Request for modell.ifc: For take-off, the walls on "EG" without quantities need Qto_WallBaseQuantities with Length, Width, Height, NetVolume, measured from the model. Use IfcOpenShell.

First a look at what the model holds.

```python
import ifcopenshell
import ifcopenshell.util.element
import ifcopenshell.util.unit

model = ifcopenshell.open("modell.ifc")
print(model.schema)
for unit_type in ("LENGTHUNIT", "AREAUNIT", "VOLUMEUNIT"):
    print(unit_type, ifcopenshell.util.unit.calculate_unit_scale(model, unit_type))
storey = next(s for s in model.by_type("IfcBuildingStorey") if s.Name == "EG")
walls = [e for e in ifcopenshell.util.element.get_decomposition(storey) if e.is_a("IfcWall")]
for e in sorted(walls, key=lambda e: e.id()):
    print(e.id(), e.is_a(), e.Name, list(ifcopenshell.util.element.get_psets(e, qtos_only=True)), sep=" | ")
```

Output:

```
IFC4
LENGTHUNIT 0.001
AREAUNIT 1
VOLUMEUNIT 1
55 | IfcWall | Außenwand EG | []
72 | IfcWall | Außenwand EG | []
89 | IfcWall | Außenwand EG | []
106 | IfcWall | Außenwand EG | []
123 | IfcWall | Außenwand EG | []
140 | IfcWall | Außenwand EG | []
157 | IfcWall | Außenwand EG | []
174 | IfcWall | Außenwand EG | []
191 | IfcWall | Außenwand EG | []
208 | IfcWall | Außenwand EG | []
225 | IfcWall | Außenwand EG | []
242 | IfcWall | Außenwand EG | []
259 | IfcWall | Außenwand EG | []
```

```python
import ifcopenshell
import ifcopenshell.api.pset
import ifcopenshell.geom
import ifcopenshell.util.element
import ifcopenshell.util.shape
import ifcopenshell.util.unit

model = ifcopenshell.open("modell.ifc")
unit_scale = ifcopenshell.util.unit.calculate_unit_scale(model)
volume_scale = ifcopenshell.util.unit.calculate_unit_scale(model, "VOLUMEUNIT")
settings = ifcopenshell.geom.settings()

storey = next(s for s in model.by_type("IfcBuildingStorey") if s.Name == "EG")
walls = [e for e in ifcopenshell.util.element.get_decomposition(storey) if e.is_a("IfcWall")]

for e in sorted(walls, key=lambda e: e.id()):
    if ifcopenshell.util.element.get_psets(e, qtos_only=True, should_inherit=False):
        continue
    # Geometry comes back in metres, in the element's own axes.
    shape = ifcopenshell.geom.create_shape(settings, e)
    values = {
        "Length": ifcopenshell.util.shape.get_x(shape.geometry) / unit_scale,
        "Width": ifcopenshell.util.shape.get_y(shape.geometry) / unit_scale,
        "Height": ifcopenshell.util.shape.get_z(shape.geometry) / unit_scale,
        "NetVolume": ifcopenshell.util.shape.get_volume(shape.geometry) / volume_scale,
    }
    qto = ifcopenshell.api.pset.add_qto(model, product=e, name="Qto_WallBaseQuantities")
    ifcopenshell.api.pset.edit_qto(model, qto=qto, properties=values)
    print(e.id(), {k: round(v, 3) for k, v in values.items()})

model.write("modell_rev.ifc")
```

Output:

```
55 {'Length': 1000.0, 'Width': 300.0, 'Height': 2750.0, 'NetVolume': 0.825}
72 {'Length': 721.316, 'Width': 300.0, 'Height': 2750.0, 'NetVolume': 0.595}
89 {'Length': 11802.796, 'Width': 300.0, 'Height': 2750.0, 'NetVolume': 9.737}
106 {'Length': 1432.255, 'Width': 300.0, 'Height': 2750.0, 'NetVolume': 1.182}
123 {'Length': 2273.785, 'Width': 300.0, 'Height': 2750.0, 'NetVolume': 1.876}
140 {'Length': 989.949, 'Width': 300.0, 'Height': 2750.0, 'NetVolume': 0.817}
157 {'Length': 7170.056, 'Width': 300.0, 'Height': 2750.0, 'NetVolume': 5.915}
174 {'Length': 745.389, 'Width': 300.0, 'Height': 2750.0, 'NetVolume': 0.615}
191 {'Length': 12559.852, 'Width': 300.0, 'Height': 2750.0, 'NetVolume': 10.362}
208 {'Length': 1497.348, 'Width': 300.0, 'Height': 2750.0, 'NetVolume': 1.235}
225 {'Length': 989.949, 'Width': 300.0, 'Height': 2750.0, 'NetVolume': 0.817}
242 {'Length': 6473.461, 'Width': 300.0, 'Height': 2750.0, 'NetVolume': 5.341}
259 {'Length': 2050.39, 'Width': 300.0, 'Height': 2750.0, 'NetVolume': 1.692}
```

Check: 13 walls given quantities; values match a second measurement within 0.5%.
